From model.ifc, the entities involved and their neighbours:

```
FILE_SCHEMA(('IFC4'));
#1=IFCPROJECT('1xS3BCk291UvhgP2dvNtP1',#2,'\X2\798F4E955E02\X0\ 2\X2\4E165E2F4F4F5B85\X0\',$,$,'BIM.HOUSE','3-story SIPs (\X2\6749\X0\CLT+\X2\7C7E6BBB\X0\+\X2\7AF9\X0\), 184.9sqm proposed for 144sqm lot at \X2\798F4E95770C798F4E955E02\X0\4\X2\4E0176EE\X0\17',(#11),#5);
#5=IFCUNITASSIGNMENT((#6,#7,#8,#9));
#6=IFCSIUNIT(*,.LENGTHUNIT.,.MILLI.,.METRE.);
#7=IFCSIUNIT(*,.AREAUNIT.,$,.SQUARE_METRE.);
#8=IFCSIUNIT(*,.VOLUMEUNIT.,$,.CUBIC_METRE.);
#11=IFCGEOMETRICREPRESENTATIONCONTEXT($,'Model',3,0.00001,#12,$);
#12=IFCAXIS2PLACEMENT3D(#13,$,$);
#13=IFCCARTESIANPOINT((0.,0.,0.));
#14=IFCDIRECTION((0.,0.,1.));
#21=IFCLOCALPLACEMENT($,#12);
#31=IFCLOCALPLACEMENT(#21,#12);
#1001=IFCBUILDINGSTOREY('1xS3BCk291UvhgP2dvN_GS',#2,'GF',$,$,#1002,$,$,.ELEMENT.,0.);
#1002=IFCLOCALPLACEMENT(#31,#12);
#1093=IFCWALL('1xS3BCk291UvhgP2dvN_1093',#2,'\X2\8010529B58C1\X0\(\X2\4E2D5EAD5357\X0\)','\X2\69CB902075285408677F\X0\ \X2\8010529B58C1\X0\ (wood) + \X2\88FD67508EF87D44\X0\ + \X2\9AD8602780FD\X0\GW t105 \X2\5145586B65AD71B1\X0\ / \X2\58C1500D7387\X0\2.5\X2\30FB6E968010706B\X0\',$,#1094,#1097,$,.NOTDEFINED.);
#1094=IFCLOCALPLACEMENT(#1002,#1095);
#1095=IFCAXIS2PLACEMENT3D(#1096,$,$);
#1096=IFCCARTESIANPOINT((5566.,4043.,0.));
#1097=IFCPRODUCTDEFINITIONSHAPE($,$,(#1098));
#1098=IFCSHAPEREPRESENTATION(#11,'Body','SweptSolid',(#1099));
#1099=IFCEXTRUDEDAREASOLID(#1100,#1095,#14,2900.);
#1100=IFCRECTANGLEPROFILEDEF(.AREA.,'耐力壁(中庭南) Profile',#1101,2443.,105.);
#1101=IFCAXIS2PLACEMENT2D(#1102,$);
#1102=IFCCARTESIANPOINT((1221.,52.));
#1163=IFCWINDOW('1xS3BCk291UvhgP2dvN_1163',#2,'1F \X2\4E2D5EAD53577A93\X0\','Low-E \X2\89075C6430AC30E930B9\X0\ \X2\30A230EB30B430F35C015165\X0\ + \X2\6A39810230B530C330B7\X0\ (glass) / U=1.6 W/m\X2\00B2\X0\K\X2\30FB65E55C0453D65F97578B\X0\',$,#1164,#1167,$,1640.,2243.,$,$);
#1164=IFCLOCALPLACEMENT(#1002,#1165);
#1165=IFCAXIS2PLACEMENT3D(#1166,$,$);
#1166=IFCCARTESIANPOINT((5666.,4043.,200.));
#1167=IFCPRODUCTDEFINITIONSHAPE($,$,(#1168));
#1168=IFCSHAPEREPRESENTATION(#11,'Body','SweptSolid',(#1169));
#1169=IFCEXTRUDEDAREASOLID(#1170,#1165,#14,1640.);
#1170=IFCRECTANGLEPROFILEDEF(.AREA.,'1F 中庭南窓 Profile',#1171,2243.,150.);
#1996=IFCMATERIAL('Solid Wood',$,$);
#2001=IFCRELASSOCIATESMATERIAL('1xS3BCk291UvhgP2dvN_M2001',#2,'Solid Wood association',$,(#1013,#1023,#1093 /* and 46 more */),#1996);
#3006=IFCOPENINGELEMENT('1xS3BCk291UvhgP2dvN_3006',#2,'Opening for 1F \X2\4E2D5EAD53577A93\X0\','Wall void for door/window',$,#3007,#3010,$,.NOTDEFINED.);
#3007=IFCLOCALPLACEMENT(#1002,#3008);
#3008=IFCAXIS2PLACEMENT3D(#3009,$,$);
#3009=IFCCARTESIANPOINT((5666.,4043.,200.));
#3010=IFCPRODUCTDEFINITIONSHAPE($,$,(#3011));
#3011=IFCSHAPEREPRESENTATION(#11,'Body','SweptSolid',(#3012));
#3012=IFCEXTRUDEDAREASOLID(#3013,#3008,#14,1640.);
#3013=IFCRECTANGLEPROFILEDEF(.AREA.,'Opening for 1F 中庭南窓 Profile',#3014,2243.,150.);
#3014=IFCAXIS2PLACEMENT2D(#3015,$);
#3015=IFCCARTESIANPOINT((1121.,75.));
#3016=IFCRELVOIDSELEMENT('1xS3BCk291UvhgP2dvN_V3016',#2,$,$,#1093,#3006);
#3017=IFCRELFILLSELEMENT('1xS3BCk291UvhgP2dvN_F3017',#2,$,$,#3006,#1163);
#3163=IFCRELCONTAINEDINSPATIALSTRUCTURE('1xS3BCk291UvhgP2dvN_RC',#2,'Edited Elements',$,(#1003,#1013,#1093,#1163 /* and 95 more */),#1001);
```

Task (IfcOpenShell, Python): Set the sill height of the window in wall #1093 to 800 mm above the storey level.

```python
import numpy as np
import ifcopenshell
import ifcopenshell.api.geometry
import ifcopenshell.geom
import ifcopenshell.util.element
import ifcopenshell.util.placement
import ifcopenshell.util.shape
import ifcopenshell.util.unit

model = ifcopenshell.open("model.ifc")
unit_scale = ifcopenshell.util.unit.calculate_unit_scale(model)

window = model.by_guid("1xS3BCk291UvhgP2dvN_1163")
opening = window.FillsVoids[0].RelatingOpeningElement
storey = ifcopenshell.util.element.get_container(window, ifc_class="IfcBuildingStorey")
level = ifcopenshell.util.placement.get_local_placement(storey.ObjectPlacement)[2, 3]

# The opening's origin need not be at the sill, so measure its lowest point.
shape = ifcopenshell.geom.create_shape(ifcopenshell.geom.settings(), opening)
bottom = ifcopenshell.util.shape.get_shape_bottom_elevation(shape, shape.geometry) / unit_scale
dz = level + 800.0 - bottom

shift = np.array([0.0, 0.0, dz])
# The window is not placed relative to its opening, so move both.
for product in (opening, window):
    matrix = ifcopenshell.util.placement.get_local_placement(product.ObjectPlacement)
    matrix[:3, 3] += shift
    ifcopenshell.api.geometry.edit_object_placement(model, product=product, matrix=matrix, is_si=False)

print(f"moved by {dz * unit_scale:+.3f} m")

model.write("model_edited.ifc")
```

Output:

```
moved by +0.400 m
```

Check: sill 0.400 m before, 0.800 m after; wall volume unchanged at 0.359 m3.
